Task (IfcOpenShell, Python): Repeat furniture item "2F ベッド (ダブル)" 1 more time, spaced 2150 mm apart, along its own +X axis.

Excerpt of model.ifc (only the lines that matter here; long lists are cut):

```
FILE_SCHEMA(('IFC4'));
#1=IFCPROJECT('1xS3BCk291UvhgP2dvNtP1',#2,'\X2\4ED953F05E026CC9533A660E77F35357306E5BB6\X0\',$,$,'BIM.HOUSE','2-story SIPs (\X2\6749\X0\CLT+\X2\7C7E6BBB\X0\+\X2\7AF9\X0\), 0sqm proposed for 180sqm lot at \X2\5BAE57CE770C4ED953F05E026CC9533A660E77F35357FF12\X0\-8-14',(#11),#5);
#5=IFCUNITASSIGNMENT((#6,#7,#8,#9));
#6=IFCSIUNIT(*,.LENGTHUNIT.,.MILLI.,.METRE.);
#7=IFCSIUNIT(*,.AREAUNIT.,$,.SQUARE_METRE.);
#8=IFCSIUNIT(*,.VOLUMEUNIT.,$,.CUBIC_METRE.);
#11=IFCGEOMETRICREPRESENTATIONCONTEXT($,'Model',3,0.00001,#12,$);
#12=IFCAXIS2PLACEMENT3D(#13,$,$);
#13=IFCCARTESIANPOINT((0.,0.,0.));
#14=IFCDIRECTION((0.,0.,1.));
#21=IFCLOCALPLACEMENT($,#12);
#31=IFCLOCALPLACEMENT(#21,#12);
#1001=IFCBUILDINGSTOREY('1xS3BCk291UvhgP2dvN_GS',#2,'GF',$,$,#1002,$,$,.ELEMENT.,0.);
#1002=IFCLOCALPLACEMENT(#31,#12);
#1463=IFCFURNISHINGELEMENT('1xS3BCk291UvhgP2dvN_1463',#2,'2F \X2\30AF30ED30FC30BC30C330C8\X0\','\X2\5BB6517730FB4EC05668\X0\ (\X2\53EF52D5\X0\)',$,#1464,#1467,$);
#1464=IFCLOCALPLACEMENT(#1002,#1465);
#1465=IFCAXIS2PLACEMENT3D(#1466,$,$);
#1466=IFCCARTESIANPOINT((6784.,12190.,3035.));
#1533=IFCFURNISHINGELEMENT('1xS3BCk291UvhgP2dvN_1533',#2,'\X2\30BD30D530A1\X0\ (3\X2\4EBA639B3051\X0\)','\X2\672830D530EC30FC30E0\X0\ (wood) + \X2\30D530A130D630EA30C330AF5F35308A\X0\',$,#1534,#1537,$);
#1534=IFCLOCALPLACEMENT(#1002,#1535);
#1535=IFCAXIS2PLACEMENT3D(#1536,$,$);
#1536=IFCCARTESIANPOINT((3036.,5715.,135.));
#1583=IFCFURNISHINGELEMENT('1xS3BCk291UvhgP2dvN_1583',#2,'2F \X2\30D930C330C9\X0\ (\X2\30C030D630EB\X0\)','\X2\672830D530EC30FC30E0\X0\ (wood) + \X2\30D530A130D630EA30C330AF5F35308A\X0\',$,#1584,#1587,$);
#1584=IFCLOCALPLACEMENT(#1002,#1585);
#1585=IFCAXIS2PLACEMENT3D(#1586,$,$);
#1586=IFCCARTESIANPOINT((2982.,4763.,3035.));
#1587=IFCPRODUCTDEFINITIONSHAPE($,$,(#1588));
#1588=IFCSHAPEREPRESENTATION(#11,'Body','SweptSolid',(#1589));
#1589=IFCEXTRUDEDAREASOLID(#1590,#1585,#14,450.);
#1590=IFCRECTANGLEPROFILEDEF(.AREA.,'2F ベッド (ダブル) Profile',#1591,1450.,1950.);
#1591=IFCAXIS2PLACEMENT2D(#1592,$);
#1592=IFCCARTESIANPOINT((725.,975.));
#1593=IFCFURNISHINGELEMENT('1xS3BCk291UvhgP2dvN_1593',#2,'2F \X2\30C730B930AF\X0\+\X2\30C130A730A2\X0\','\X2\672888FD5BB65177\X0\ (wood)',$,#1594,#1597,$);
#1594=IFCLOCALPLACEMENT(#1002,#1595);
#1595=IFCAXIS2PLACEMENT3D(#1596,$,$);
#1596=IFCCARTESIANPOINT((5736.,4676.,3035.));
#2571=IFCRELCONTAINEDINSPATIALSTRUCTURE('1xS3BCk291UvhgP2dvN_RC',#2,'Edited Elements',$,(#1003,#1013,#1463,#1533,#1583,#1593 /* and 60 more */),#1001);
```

```python
import ifcopenshell
import ifcopenshell.api.geometry
import ifcopenshell.api.root
import ifcopenshell.util.element
import ifcopenshell.util.placement

model = ifcopenshell.open("model.ifc")


def reuse_history(source, copy):
    """copy_class also copies each property set's owner history, people and application; keep the originals."""
    for rel in copy.IsDefinedBy:
        if rel.is_a("IfcRelDefinesByProperties") and (history := rel.RelatingPropertyDefinition.OwnerHistory):
            rel.RelatingPropertyDefinition.OwnerHistory = source.OwnerHistory
            ifcopenshell.util.element.remove_deep2(model, history)


source = model.by_guid("1xS3BCk291UvhgP2dvN_1583")
base = ifcopenshell.util.placement.get_local_placement(source.ObjectPlacement)
step = base[:3, 0] * 2150.0

for i in range(1, 2):
    copy = ifcopenshell.api.root.copy_class(model, product=source)
    copy.Representation = ifcopenshell.util.element.copy_deep(
        model, source.Representation, exclude=["IfcGeometricRepresentationContext", "IfcRepresentationMap"]
    )
    reuse_history(source, copy)
    matrix = base.copy()
    matrix[:3, 3] += i * step
    print("added at", matrix[:3, 3].round(3) + 0.0)
    ifcopenshell.api.geometry.edit_object_placement(model, product=copy, matrix=matrix, is_si=False)

model.write("model_rev.ifc")
```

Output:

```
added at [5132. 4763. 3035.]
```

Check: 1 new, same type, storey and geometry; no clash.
